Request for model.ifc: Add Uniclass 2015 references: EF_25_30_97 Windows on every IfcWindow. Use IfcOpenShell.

First a look at what the model holds.

```python
import ifcopenshell

model = ifcopenshell.open("model.ifc")
print(model.schema)
print("classifications:", [c.Name for c in model.by_type("IfcClassification")])
for ifc_class in ("IfcDoor", "IfcRoof", "IfcStair", "IfcWall", "IfcWindow"):
    print(ifc_class, len(model.by_type(ifc_class)))
```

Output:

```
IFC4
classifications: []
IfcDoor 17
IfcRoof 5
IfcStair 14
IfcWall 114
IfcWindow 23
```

```python
import ifcopenshell
import ifcopenshell.api.classification

model = ifcopenshell.open("model.ifc")

system = ifcopenshell.api.classification.add_classification(model, classification="Uniclass 2015")

codes = {
    "IfcWindow": ("EF_25_30_97", "Windows"),
}
for ifc_class, (code, name) in codes.items():
    products = model.by_type(ifc_class)
    ifcopenshell.api.classification.add_reference(
        model, products=products, classification=system, identification=code, name=name
    )
    print(code, len(products))

model.write("model-out.ifc")
```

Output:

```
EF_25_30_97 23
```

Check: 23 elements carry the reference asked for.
